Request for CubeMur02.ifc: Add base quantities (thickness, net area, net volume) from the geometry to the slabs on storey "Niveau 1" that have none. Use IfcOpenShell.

First a look at what the model holds.

```python
import ifcopenshell
import ifcopenshell.util.element
import ifcopenshell.util.unit

model = ifcopenshell.open("CubeMur02.ifc")
print(model.schema)
for unit_type in ("LENGTHUNIT", "AREAUNIT", "VOLUMEUNIT"):
    print(unit_type, ifcopenshell.util.unit.calculate_unit_scale(model, unit_type))
storey = next(s for s in model.by_type("IfcBuildingStorey") if s.Name == "Niveau 1")
slabs = [e for e in ifcopenshell.util.element.get_decomposition(storey) if e.is_a("IfcSlab")]
for e in sorted(slabs, key=lambda e: e.id()):
    print(e.id(), e.is_a(), e.Name, list(ifcopenshell.util.element.get_psets(e, qtos_only=True)), sep=" | ")
```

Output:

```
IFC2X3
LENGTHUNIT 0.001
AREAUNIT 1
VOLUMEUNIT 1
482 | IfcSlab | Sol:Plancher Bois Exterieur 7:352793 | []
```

```python
import ifcopenshell
import ifcopenshell.api.pset
import ifcopenshell.geom
import ifcopenshell.util.element
import ifcopenshell.util.shape
import ifcopenshell.util.unit

model = ifcopenshell.open("CubeMur02.ifc")
unit_scale = ifcopenshell.util.unit.calculate_unit_scale(model)
area_scale = ifcopenshell.util.unit.calculate_unit_scale(model, "AREAUNIT")
volume_scale = ifcopenshell.util.unit.calculate_unit_scale(model, "VOLUMEUNIT")
settings = ifcopenshell.geom.settings()

storey = next(s for s in model.by_type("IfcBuildingStorey") if s.Name == "Niveau 1")
slabs = [e for e in ifcopenshell.util.element.get_decomposition(storey) if e.is_a("IfcSlab")]

for e in sorted(slabs, key=lambda e: e.id()):
    if ifcopenshell.util.element.get_psets(e, qtos_only=True, should_inherit=False):
        continue
    # Geometry comes back in metres, in the element's own axes.
    shape = ifcopenshell.geom.create_shape(settings, e)
    values = {
        "Width": ifcopenshell.util.shape.get_z(shape.geometry) / unit_scale,
        "NetArea": ifcopenshell.util.shape.get_footprint_area(shape.geometry) / area_scale,
        "NetVolume": ifcopenshell.util.shape.get_volume(shape.geometry) / volume_scale,
    }
    qto = ifcopenshell.api.pset.add_qto(model, product=e, name="BaseQuantities")
    ifcopenshell.api.pset.edit_qto(model, qto=qto, properties=values)
    print(e.id(), {k: round(v, 3) for k, v in values.items()})

model.write("CubeMur02_v2.ifc")
```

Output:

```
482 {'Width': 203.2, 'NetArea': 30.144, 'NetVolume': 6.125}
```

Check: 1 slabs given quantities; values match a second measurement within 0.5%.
